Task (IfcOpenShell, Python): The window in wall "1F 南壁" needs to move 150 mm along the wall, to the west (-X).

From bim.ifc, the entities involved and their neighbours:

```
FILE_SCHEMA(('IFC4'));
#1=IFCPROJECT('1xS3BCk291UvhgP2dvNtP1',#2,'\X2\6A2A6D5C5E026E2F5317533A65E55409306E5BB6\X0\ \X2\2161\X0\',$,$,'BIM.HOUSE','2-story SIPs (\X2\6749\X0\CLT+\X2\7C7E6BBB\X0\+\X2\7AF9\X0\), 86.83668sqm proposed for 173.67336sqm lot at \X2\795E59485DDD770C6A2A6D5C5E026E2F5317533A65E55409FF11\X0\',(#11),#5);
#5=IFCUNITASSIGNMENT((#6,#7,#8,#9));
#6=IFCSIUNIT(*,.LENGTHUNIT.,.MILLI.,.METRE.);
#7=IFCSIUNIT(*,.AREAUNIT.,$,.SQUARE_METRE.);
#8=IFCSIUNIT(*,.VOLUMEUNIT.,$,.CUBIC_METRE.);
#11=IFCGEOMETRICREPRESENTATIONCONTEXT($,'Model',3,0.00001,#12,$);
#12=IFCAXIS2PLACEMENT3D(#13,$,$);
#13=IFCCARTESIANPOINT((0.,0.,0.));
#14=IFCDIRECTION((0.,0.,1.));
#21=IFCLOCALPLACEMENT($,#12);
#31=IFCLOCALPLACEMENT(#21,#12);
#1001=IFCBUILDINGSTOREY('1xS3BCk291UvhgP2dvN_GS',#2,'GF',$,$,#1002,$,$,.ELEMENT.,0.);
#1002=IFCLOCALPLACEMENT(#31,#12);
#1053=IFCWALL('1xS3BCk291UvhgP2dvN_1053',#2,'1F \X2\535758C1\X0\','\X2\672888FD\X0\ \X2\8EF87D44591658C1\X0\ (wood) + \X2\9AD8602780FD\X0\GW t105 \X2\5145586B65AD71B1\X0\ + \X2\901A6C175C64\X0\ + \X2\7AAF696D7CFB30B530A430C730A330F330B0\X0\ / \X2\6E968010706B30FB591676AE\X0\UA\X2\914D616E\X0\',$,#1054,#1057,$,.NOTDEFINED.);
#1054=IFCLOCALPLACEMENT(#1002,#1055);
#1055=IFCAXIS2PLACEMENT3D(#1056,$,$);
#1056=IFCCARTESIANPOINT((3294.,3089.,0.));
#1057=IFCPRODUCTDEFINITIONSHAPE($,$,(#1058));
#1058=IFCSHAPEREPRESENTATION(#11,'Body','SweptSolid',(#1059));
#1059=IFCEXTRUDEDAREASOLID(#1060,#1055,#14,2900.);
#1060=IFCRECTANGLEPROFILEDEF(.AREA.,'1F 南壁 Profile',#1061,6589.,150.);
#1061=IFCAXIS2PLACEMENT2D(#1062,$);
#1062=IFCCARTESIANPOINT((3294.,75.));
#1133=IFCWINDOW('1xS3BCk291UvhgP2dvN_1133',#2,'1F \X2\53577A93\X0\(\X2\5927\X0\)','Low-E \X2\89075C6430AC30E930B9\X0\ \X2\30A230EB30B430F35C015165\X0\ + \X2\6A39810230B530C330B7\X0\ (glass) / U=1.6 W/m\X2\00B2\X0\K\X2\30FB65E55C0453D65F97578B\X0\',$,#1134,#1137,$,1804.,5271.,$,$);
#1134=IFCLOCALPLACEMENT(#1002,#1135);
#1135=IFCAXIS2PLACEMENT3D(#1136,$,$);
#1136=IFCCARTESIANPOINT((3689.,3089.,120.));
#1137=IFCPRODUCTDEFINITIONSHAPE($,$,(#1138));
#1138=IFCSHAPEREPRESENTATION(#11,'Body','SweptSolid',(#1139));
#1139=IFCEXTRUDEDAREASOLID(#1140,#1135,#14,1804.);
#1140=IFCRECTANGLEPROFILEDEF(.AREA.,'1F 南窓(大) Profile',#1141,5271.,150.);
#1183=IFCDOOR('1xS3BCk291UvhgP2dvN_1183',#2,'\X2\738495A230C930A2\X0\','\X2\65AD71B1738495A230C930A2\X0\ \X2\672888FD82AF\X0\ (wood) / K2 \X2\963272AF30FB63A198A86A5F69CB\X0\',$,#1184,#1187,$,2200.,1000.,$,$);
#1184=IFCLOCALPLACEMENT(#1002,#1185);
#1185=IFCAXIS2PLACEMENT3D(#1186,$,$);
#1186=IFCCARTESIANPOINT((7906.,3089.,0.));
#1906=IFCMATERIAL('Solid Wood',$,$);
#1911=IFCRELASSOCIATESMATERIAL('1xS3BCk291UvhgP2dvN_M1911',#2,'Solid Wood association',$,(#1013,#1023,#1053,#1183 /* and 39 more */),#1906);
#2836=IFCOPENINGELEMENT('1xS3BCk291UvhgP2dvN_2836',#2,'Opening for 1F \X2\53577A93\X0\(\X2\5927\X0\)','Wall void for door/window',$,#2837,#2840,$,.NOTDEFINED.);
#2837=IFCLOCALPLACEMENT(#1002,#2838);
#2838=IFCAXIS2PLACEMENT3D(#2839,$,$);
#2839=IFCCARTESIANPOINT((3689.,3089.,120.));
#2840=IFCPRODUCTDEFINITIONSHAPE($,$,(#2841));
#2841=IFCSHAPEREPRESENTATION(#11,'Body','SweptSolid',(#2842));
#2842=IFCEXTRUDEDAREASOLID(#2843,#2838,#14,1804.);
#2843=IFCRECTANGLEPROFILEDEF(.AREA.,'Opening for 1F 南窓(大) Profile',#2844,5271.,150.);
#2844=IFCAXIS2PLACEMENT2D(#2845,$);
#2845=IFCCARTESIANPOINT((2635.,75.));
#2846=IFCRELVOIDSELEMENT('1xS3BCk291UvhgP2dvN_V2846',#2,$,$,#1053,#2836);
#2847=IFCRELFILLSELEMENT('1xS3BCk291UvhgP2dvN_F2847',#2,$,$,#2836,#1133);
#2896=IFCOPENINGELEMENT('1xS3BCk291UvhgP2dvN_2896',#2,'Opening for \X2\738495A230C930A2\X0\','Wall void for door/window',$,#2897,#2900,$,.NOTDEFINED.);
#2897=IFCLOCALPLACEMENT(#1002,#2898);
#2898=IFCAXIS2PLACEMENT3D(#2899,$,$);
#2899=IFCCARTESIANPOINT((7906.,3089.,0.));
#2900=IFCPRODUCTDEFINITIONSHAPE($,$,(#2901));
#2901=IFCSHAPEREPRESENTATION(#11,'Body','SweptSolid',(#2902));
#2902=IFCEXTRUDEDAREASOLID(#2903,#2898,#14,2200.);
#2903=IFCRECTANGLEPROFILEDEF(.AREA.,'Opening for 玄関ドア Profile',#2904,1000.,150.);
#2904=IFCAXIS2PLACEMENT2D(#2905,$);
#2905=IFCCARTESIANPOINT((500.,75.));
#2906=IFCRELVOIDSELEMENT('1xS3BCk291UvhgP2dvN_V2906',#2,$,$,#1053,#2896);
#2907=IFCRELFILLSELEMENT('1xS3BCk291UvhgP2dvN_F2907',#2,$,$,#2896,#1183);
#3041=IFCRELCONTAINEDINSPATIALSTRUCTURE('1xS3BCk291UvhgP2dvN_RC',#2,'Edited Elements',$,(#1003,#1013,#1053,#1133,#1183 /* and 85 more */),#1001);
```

```python
import ifcopenshell
import ifcopenshell.api.geometry
import ifcopenshell.util.placement

model = ifcopenshell.open("bim.ifc")

window = model.by_guid("1xS3BCk291UvhgP2dvN_1133")
opening = window.FillsVoids[0].RelatingOpeningElement
wall = opening.VoidsElements[0].RelatingBuildingElement

wall_matrix = ifcopenshell.util.placement.get_local_placement(wall.ObjectPlacement)
shift = wall_matrix[:3, 0] * -150.0
before = ifcopenshell.util.placement.get_local_placement(window.ObjectPlacement)[:3, 3].copy()

# The window is not placed relative to its opening, so move both.
for product in (opening, window):
    matrix = ifcopenshell.util.placement.get_local_placement(product.ObjectPlacement)
    matrix[:3, 3] += shift
    ifcopenshell.api.geometry.edit_object_placement(model, product=product, matrix=matrix, is_si=False)

after = ifcopenshell.util.placement.get_local_placement(window.ObjectPlacement)[:3, 3]
print("window moved by", (after - before).round(3) + 0.0)

model.write("bim_edited.ifc")
```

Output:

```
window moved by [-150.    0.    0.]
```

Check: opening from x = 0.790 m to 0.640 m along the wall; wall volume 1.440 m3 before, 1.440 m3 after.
